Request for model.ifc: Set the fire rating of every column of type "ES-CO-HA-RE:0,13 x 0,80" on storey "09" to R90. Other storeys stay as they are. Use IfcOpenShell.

First a look at what the model holds.

```python
import ifcopenshell
import ifcopenshell.util.element

model = ifcopenshell.open("model.ifc")
print(model.schema)
storey = next(s for s in model.by_type("IfcBuildingStorey") if s.Name == "09")
columns = [e for e in ifcopenshell.util.element.get_decomposition(storey) if e.is_a("IfcColumn")]
seen = {}
for e in columns:
    element_type = ifcopenshell.util.element.get_type(e)
    key = (element_type.Name if element_type != e and element_type else None, ifcopenshell.util.element.get_pset(e, "Pset_ColumnCommon", "FireRating"))
    seen[key] = seen.get(key, 0) + 1
for (name, value), count in sorted(seen.items(), key=str):
    print(count, "x", name, "|", value)
```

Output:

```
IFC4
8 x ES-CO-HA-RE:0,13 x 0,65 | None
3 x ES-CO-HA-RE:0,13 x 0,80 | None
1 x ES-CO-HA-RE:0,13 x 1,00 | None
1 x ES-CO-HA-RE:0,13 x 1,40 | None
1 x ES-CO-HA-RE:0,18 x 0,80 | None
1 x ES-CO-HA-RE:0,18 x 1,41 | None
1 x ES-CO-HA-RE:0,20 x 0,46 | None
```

```python
import ifcopenshell
import ifcopenshell.api.pset
import ifcopenshell.util.element

model = ifcopenshell.open("model.ifc")

storey = next(s for s in model.by_type("IfcBuildingStorey") if s.Name == "09")
columns = [e for e in ifcopenshell.util.element.get_decomposition(storey) if e.is_a("IfcColumn")]

count = 0
for e in columns:
    element_type = ifcopenshell.util.element.get_type(e)
    if element_type in (None, e) or element_type.Name != "ES-CO-HA-RE:0,13 x 0,80":
        continue
    # add_pset returns the element's existing set when there is one.
    pset = ifcopenshell.api.pset.add_pset(model, product=e, name="Pset_ColumnCommon")
    ifcopenshell.api.pset.edit_pset(model, pset=pset, properties={"FireRating": "R90"})
    count += 1

print(count, "columns updated")

model.write("model_v2.ifc")
```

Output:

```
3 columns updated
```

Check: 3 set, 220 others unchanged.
